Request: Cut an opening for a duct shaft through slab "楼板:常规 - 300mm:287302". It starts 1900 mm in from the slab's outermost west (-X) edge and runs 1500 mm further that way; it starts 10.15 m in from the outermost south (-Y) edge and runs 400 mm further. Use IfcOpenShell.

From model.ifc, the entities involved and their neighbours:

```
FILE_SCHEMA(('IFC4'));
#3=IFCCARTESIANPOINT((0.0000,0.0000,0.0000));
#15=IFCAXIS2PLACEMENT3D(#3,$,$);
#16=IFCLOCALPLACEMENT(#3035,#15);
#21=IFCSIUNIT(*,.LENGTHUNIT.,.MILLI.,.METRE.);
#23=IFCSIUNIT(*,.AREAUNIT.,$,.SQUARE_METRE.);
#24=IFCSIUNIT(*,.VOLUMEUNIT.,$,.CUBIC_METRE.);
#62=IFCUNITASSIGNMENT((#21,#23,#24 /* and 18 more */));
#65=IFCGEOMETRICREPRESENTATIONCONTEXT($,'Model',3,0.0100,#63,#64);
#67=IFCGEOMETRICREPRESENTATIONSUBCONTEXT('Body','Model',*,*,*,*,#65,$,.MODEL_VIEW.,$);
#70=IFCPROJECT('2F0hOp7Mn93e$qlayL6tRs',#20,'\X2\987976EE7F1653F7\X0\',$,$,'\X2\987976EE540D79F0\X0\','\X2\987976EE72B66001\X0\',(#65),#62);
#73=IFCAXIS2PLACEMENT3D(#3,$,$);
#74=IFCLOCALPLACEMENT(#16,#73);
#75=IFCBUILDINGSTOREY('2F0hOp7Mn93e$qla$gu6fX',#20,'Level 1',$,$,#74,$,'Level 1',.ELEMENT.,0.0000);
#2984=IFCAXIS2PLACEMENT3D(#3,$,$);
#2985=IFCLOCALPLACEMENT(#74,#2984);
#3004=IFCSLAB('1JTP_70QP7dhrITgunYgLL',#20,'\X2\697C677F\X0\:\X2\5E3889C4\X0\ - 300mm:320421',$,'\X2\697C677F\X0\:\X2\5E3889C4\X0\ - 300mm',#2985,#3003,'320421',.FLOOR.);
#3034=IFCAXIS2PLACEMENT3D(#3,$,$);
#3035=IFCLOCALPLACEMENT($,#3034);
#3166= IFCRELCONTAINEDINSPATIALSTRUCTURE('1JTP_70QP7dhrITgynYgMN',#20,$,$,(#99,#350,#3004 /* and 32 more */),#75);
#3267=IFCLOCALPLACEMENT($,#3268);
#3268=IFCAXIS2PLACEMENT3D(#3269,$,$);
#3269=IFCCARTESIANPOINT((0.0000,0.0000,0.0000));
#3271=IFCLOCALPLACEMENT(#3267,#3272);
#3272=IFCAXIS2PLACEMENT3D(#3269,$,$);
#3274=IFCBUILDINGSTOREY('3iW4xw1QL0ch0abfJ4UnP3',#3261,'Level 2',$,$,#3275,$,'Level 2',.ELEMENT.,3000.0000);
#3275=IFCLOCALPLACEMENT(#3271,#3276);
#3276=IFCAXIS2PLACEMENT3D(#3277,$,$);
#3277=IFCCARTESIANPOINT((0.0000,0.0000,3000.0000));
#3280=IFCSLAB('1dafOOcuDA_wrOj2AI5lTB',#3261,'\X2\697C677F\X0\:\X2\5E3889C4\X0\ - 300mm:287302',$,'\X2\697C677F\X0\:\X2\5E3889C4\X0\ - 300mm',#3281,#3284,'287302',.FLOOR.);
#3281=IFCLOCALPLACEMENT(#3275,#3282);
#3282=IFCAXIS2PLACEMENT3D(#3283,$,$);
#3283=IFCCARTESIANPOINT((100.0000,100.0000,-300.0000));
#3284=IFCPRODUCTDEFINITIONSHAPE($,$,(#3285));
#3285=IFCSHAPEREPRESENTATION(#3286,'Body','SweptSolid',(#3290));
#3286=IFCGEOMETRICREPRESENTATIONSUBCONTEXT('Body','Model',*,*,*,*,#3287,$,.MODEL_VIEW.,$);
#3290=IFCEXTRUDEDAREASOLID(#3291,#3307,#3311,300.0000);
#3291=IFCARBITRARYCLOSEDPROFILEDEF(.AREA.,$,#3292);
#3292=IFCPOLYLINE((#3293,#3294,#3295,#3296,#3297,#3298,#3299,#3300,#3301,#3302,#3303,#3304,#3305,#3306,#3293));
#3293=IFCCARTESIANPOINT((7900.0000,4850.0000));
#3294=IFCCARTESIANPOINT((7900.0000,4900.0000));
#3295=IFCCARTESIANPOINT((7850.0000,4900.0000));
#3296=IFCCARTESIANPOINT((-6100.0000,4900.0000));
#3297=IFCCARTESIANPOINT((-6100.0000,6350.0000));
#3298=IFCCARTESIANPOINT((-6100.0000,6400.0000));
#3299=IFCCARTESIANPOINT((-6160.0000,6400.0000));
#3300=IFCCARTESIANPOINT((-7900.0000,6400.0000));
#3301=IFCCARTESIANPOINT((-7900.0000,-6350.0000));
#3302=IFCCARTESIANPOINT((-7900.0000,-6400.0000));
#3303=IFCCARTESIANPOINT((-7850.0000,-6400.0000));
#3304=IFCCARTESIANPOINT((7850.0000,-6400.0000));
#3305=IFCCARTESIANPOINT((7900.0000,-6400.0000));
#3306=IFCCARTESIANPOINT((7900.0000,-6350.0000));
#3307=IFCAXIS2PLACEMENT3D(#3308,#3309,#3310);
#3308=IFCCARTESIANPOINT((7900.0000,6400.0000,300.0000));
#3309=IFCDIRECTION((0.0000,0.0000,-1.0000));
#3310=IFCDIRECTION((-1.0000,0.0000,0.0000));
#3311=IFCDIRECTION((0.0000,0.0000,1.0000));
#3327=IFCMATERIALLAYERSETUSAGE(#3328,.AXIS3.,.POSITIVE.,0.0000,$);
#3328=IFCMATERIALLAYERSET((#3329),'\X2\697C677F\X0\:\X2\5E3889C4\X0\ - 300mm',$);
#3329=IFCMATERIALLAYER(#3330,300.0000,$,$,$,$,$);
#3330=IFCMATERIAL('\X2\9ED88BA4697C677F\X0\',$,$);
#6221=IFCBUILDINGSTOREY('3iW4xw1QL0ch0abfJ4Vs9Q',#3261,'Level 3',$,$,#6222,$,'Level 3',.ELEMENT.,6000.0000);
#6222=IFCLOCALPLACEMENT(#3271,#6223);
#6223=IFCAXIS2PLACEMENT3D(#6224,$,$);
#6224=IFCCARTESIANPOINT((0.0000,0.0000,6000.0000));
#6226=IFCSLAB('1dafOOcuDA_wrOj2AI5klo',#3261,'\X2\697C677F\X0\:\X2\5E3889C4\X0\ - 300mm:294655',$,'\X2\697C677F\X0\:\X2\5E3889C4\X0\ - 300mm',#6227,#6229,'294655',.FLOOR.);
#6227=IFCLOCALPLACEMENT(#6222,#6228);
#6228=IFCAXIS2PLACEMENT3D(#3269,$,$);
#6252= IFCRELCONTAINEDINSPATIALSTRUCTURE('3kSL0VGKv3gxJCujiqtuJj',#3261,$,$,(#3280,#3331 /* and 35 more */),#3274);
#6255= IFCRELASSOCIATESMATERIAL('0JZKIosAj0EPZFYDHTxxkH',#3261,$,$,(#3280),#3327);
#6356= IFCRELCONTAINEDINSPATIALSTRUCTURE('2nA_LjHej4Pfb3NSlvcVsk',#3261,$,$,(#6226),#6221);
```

```python
import numpy as np
import ifcopenshell
import ifcopenshell.api.feature
import ifcopenshell.api.geometry
import ifcopenshell.api.root
import ifcopenshell.geom
import ifcopenshell.util.placement
import ifcopenshell.util.representation
import ifcopenshell.util.shape
import ifcopenshell.util.unit

model = ifcopenshell.open("model.ifc")
unit_scale = ifcopenshell.util.unit.calculate_unit_scale(model)
settings = ifcopenshell.geom.settings()


def volume(element):
    """Net volume in cubic metres, openings subtracted."""
    shape = ifcopenshell.geom.create_shape(settings, element)
    return ifcopenshell.util.shape.get_volume(shape.geometry)


slab = model.by_guid("1dafOOcuDA_wrOj2AI5lTB")
before = volume(slab)

# Extent in the slab's own axes, in metres. The edges named are its -X and -Y sides.
slab_shape = ifcopenshell.geom.create_shape(settings, slab)
vertices = ifcopenshell.util.shape.get_vertices(slab_shape.geometry)
x_min, y_min, bottom = vertices.min(axis=0)
top = vertices[:, 2].max()

opening = ifcopenshell.api.root.create_entity(model, ifc_class="IfcOpeningElement", name="Duct shaft opening", predefined_type="OPENING")
context = ifcopenshell.util.representation.get_context(model, "Model", "Body", "MODEL_VIEW")
width, depth = 1.5, 0.4
outline = [(0.0, 0.0), (width, 0.0), (width, depth), (0.0, depth), (0.0, 0.0)]
# Overshoot both faces by 50 mm so the cut is clean.
shape = ifcopenshell.api.geometry.add_slab_representation(
    model, context=context, depth=top - bottom + 0.1, polyline=outline
)
ifcopenshell.api.geometry.assign_representation(model, product=opening, representation=shape)

matrix = ifcopenshell.util.placement.get_local_placement(slab.ObjectPlacement)
matrix[:, 3] = matrix @ np.append(np.array([x_min + 1.9, y_min + 10.15, bottom - 0.05]) / unit_scale, 1.0)
ifcopenshell.api.geometry.edit_object_placement(model, product=opening, matrix=matrix, is_si=False)
ifcopenshell.api.feature.add_feature(model, feature=opening, element=slab)

after = volume(slab)

print(f"slab volume {before:.3f} -> {after:.3f} m3")

model.write("model_updated.ifc")
```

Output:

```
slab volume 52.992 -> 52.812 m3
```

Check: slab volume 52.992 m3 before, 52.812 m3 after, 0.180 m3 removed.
